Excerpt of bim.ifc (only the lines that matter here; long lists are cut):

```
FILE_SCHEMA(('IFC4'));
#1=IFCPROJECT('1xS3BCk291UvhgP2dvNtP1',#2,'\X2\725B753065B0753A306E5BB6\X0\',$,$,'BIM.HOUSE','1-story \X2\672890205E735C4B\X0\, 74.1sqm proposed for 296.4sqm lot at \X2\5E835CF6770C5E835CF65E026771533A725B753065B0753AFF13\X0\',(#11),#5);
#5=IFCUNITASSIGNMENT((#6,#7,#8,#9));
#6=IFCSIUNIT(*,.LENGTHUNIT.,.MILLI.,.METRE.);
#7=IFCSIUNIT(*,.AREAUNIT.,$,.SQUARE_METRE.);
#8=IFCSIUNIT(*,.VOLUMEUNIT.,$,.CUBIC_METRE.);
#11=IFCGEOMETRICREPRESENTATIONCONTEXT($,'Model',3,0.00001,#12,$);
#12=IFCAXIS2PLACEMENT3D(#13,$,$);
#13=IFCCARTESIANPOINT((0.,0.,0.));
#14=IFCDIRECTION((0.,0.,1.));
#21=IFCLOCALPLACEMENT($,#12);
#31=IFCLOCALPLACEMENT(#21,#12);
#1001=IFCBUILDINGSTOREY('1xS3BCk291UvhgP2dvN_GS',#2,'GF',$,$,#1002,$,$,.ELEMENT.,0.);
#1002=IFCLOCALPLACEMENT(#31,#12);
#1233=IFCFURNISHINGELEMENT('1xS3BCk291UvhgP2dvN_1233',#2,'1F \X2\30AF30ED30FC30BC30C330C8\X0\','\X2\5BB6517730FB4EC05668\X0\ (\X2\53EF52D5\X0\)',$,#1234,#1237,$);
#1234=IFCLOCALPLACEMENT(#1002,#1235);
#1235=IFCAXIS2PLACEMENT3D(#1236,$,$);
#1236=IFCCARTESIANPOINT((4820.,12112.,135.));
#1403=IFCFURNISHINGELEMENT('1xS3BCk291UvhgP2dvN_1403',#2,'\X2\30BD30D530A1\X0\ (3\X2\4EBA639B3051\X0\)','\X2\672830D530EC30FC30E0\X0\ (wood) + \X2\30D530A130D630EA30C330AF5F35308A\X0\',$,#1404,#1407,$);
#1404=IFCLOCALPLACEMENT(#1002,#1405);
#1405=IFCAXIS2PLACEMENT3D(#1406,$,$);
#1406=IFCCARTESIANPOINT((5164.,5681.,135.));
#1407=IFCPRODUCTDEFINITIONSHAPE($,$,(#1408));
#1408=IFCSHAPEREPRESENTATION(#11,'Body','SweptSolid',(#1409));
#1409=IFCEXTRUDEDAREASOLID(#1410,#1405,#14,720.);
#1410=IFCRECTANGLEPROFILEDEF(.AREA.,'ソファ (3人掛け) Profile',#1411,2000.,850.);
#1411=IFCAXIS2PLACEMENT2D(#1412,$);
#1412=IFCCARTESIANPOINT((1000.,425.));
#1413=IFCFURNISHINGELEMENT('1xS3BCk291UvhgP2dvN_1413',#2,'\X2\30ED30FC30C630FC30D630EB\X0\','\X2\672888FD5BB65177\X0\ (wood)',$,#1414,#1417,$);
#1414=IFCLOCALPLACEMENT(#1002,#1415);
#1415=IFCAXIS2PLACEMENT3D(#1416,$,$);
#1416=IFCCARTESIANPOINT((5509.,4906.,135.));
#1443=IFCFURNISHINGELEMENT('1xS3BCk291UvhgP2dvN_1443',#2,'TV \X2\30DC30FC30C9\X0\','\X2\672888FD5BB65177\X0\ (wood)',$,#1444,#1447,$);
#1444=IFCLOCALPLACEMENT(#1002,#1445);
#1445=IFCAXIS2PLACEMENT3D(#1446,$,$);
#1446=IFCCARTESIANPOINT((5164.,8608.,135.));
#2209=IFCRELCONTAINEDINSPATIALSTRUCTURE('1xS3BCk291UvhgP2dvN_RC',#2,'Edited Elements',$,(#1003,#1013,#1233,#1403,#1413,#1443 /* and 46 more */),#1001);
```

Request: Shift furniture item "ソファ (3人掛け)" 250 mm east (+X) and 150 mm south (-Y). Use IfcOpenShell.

```python
import ifcopenshell
import ifcopenshell.api.geometry
import ifcopenshell.util.placement

model = ifcopenshell.open("bim.ifc")

item = model.by_guid("1xS3BCk291UvhgP2dvN_1403")
matrix = ifcopenshell.util.placement.get_local_placement(item.ObjectPlacement)
matrix[0, 3] += 250.0
matrix[1, 3] -= 150.0
ifcopenshell.api.geometry.edit_object_placement(model, product=item, matrix=matrix, is_si=False)

print(ifcopenshell.util.placement.get_local_placement(item.ObjectPlacement).round(3) + 0.0)

model.write("bim_updated.ifc")
```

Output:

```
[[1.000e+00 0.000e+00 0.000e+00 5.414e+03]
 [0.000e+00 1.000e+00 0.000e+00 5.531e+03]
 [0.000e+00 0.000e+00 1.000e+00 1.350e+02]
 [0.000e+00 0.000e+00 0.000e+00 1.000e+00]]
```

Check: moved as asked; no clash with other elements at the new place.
